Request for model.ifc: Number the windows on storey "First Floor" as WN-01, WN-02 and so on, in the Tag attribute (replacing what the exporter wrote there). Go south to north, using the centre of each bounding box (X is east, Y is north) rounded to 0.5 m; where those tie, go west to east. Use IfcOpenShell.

First a look at what the model holds.

```python
import ifcopenshell
import ifcopenshell.util.element
import ifcopenshell.util.placement

model = ifcopenshell.open("model.ifc")
print(model.schema)
storey = next(s for s in model.by_type("IfcBuildingStorey") if s.Name == "First Floor")
windows = [e for e in ifcopenshell.util.element.get_decomposition(storey) if e.is_a("IfcWindow")]
for e in sorted(windows, key=lambda e: e.id()):
    origin = ifcopenshell.util.placement.get_local_placement(e.ObjectPlacement)[:3, 3]
    print(e.id(), e.Tag, e.Name, origin.round(2) + 0.0, sep=" | ")
```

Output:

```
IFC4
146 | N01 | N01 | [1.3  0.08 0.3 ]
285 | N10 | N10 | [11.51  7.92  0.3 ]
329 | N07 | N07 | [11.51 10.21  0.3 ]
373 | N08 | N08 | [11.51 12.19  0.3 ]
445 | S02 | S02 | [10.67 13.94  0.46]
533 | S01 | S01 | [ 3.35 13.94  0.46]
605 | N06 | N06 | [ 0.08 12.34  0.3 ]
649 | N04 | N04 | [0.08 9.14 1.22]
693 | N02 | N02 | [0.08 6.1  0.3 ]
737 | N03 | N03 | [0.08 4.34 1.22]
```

```python
import ifcopenshell
import ifcopenshell.geom
import ifcopenshell.util.element
import ifcopenshell.util.shape

model = ifcopenshell.open("model.ifc")
settings = ifcopenshell.geom.settings()
settings.set("use-world-coords", True)


def centre(element):
    shape = ifcopenshell.geom.create_shape(settings, element)
    return ifcopenshell.util.shape.get_bbox_centroid(shape.geometry)


storey = next(s for s in model.by_type("IfcBuildingStorey") if s.Name == "First Floor")
windows = [e for e in ifcopenshell.util.element.get_decomposition(storey) if e.is_a("IfcWindow")]

# Insertion points can sit at a corner or the storey origin, so sort by the geometry (in metres).
centres = {e: centre(e) for e in windows}
windows.sort(key=lambda e: (round(centres[e][1] / 0.5), centres[e][0]))

for i, e in enumerate(windows, start=1):
    number = f"WN-{i:02d}"
    e.Tag = number
    print(e.id(), number)

model.write("model_v2.ifc")
```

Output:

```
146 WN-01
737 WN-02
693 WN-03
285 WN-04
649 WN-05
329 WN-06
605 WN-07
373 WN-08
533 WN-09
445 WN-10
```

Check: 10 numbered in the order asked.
